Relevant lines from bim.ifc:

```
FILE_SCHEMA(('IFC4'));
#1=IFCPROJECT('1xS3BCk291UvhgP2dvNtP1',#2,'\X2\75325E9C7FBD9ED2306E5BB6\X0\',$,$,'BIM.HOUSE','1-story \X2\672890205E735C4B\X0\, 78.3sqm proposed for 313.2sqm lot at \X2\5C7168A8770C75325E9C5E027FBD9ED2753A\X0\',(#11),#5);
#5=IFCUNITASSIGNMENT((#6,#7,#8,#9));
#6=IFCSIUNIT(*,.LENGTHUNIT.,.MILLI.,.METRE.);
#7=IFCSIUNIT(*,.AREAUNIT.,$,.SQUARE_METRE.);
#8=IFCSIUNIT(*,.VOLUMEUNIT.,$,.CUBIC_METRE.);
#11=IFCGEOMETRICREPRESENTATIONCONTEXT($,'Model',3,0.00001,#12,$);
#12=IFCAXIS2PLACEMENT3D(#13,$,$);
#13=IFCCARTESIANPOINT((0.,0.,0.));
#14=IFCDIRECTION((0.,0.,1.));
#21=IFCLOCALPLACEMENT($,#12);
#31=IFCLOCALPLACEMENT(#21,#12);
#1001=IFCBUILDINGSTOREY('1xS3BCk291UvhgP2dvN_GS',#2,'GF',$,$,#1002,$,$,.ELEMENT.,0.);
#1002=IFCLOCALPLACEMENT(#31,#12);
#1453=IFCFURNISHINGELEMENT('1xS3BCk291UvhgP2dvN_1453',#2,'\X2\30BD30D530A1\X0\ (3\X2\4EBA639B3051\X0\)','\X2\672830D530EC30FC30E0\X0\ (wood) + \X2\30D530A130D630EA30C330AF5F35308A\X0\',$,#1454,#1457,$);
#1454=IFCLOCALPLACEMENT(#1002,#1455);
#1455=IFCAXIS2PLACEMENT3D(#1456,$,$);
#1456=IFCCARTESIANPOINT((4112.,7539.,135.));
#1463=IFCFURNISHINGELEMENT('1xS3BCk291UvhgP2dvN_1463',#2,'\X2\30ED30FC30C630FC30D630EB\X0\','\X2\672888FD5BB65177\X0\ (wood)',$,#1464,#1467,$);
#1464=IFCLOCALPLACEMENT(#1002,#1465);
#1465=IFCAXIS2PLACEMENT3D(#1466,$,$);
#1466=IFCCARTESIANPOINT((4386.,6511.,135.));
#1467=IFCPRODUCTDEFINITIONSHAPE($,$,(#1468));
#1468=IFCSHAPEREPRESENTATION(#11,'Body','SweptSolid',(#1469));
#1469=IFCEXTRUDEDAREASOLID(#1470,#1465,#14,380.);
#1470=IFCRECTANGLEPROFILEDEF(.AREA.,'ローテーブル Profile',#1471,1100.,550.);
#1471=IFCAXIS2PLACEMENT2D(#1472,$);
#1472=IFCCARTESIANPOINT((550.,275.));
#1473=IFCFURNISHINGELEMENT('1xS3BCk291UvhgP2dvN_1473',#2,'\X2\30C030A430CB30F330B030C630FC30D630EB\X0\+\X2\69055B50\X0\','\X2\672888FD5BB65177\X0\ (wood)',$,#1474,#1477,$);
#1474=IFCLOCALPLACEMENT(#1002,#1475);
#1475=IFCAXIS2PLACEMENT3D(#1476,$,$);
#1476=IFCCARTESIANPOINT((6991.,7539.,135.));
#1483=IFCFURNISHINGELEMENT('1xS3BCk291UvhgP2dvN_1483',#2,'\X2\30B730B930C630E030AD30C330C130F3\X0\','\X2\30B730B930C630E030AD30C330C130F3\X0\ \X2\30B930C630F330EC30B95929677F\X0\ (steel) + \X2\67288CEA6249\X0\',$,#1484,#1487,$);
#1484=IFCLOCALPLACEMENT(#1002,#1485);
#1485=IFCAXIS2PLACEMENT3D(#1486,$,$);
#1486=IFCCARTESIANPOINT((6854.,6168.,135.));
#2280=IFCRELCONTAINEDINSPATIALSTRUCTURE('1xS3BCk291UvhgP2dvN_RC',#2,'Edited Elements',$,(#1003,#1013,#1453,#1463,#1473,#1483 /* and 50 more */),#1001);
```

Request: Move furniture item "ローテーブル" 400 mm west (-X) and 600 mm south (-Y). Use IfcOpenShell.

```python
import ifcopenshell
import ifcopenshell.api.geometry
import ifcopenshell.util.placement
import ifcopenshell.util.unit

model = ifcopenshell.open("bim.ifc")
unit_scale = ifcopenshell.util.unit.calculate_unit_scale(model)

item = model.by_guid("1xS3BCk291UvhgP2dvN_1463")
matrix = ifcopenshell.util.placement.get_local_placement(item.ObjectPlacement)
matrix[0, 3] -= 0.4 / unit_scale
matrix[1, 3] -= 0.6 / unit_scale
ifcopenshell.api.geometry.edit_object_placement(model, product=item, matrix=matrix, is_si=False)

print(ifcopenshell.util.placement.get_local_placement(item.ObjectPlacement).round(3) + 0.0)

model.write("bim_v2.ifc")
```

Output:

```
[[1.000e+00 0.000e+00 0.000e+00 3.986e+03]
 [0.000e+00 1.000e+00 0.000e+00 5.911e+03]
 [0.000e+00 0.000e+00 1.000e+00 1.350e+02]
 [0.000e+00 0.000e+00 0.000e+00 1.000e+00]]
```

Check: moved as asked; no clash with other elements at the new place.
